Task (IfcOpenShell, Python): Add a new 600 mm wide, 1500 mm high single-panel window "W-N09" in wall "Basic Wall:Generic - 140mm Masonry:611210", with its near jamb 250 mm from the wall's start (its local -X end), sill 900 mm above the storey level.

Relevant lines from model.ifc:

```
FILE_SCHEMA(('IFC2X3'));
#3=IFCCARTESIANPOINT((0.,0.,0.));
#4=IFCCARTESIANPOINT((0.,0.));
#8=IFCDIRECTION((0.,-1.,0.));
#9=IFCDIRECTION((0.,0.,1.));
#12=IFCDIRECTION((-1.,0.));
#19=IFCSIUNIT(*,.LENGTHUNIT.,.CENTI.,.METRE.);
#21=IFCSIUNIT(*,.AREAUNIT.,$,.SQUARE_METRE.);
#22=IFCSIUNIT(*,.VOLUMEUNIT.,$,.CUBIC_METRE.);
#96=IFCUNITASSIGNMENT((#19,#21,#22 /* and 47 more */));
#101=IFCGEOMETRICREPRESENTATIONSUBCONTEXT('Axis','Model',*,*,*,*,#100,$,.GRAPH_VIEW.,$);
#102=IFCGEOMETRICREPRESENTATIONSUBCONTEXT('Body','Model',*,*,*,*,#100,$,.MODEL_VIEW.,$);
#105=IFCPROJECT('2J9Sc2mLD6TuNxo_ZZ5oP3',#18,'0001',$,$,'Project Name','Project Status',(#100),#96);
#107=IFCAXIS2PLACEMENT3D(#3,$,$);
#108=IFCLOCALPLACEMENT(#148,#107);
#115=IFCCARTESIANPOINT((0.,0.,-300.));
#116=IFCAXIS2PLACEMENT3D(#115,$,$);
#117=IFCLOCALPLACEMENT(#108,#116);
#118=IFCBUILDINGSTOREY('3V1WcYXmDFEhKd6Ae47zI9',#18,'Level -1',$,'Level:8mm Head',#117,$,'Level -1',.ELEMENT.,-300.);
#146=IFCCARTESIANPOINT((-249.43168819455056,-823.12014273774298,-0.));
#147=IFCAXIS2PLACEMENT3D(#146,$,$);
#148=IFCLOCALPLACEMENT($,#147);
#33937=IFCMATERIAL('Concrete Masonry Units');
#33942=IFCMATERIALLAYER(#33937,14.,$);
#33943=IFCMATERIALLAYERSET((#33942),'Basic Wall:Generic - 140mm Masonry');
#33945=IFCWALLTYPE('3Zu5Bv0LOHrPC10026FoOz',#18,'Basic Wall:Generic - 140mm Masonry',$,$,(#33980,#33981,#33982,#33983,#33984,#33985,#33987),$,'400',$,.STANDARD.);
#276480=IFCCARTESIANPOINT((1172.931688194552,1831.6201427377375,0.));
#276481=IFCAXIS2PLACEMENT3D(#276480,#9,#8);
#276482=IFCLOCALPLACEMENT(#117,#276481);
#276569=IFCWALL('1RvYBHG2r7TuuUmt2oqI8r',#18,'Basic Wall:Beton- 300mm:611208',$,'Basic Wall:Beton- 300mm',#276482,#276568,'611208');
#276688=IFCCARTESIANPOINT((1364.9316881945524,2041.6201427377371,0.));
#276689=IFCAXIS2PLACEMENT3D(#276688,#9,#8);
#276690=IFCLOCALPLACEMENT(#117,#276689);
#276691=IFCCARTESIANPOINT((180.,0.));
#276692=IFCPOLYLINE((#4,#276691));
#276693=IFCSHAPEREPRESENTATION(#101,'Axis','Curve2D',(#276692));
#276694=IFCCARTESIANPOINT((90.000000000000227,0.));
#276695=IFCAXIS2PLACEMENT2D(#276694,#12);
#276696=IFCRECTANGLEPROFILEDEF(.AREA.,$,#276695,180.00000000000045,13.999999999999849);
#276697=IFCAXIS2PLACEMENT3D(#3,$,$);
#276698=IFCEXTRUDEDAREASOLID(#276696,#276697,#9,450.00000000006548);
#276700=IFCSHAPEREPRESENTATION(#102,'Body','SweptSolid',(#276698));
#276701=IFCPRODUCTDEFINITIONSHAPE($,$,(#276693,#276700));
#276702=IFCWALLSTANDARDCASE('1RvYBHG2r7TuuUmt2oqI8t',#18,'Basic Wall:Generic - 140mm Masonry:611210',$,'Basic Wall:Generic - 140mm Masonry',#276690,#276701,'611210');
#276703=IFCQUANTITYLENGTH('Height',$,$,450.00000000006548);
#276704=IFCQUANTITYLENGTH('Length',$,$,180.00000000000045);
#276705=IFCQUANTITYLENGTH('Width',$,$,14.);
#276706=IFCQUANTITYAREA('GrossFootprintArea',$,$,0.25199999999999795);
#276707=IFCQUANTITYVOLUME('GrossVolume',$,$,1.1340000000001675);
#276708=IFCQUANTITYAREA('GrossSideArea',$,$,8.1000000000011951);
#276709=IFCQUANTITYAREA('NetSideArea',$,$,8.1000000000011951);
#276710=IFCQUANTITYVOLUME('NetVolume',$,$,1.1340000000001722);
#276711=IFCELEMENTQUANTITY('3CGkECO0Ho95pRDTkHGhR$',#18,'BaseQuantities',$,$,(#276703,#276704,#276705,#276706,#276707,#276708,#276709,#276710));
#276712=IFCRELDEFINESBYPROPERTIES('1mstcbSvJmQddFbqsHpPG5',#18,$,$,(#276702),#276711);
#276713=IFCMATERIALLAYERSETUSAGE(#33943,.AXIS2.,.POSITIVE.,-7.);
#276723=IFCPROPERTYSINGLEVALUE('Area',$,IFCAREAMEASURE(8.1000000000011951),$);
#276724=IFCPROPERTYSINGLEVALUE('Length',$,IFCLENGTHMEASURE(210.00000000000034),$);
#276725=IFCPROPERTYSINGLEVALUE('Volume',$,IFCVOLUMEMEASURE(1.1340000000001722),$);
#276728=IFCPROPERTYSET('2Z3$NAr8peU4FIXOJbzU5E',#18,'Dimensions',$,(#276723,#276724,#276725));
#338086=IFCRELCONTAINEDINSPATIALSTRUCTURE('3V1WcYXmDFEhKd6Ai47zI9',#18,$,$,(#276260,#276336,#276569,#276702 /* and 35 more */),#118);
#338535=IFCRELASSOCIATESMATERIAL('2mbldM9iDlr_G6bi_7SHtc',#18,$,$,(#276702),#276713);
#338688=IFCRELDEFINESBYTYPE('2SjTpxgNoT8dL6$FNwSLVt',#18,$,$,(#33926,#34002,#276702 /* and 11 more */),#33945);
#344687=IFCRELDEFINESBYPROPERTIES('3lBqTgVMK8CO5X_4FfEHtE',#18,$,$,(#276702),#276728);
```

```python
import numpy as np
import ifcopenshell
import ifcopenshell.api.feature
import ifcopenshell.api.geometry
import ifcopenshell.api.pset
import ifcopenshell.api.root
import ifcopenshell.api.spatial
import ifcopenshell.api.type
import ifcopenshell.geom
import ifcopenshell.util.element
import ifcopenshell.util.placement
import ifcopenshell.util.representation
import ifcopenshell.util.shape
import ifcopenshell.util.unit

model = ifcopenshell.open("model.ifc")
unit_scale = ifcopenshell.util.unit.calculate_unit_scale(model)
area_scale = ifcopenshell.util.unit.calculate_unit_scale(model, "AREAUNIT")
volume_scale = ifcopenshell.util.unit.calculate_unit_scale(model, "VOLUMEUNIT")
settings = ifcopenshell.geom.settings()


def volume(element):
    """Net volume in cubic metres, openings subtracted."""
    shape = ifcopenshell.geom.create_shape(settings, element)
    return ifcopenshell.util.shape.get_volume(shape.geometry)


wall = model.by_id(276702)
storey = ifcopenshell.util.element.get_container(wall, ifc_class="IfcBuildingStorey")
context = ifcopenshell.util.representation.get_context(model, "Model", "Body", "MODEL_VIEW")
before = volume(wall)

width, height, from_end, sill = 0.6, 1.5, 0.25, 0.9  # metres

# The wall runs along its own X axis, and the end named is its -X end.
wall_shape = ifcopenshell.geom.create_shape(settings, wall)
x, y, z = ifcopenshell.util.shape.get_vertices(wall_shape.geometry).T
start = x.min() + from_end
face, thickness = float(y.min()), float(y.max() - y.min())
wall_matrix = ifcopenshell.util.placement.get_local_placement(wall.ObjectPlacement)
level = ifcopenshell.util.placement.get_local_placement(storey.ObjectPlacement)[2, 3]


def in_wall(x, y):
    """Placement at x, y metres in the wall's axes, at sill height."""
    matrix = wall_matrix.copy()
    matrix[:, 3] = wall_matrix @ np.array([x / unit_scale, y / unit_scale, 0.0, 1.0])
    matrix[2, 3] = level + sill / unit_scale
    return matrix


# Opening: a box that overshoots both wall faces by 50 mm.
opening = ifcopenshell.api.root.create_entity(model, ifc_class="IfcOpeningElement")
box = ifcopenshell.api.geometry.add_wall_representation(
    model, context=context, length=width, height=height, thickness=thickness + 0.1
)
ifcopenshell.api.geometry.assign_representation(model, product=opening, representation=box)
ifcopenshell.api.geometry.edit_object_placement(model, product=opening, matrix=in_wall(start, face - 0.05), is_si=False)
ifcopenshell.api.feature.add_feature(model, feature=opening, element=wall)

window = ifcopenshell.api.root.create_entity(model, ifc_class="IfcWindow", name="W-N09")
window.OverallWidth, window.OverallHeight = width / unit_scale, height / unit_scale
body = ifcopenshell.api.geometry.add_window_representation(
    model,
    context=context,
    overall_width=window.OverallWidth,
    overall_height=window.OverallHeight,
    partition_type="SINGLE_PANEL",
)
ifcopenshell.api.geometry.assign_representation(model, product=window, representation=body)
ifcopenshell.api.spatial.assign_container(model, products=[window], relating_structure=storey)
fills = ifcopenshell.api.feature.add_filling(model, opening=opening, element=window)
fills.OwnerHistory = window.OwnerHistory  # required in IFC2X3

# IFC2X3 keeps the operation on the window style.
style = ifcopenshell.api.root.create_entity(model, ifc_class="IfcWindowStyle", name="W-N09")
style.OperationType, style.ConstructionType = "SINGLE_PANEL", "NOTDEFINED"
style.ParameterTakesPrecedence = style.Sizeable = False
ifcopenshell.api.type.assign_type(model, related_objects=[window], relating_type=style)

# Centre the window in the wall's thickness.
ifcopenshell.api.geometry.edit_object_placement(model, product=window, matrix=in_wall(start, face), is_si=False)
window_shape = ifcopenshell.geom.create_shape(settings, window)
depth = ifcopenshell.util.shape.get_vertices(window_shape.geometry)[:, 1]
offset = face + thickness / 2 - (depth.min() + depth.max()) / 2
ifcopenshell.api.geometry.edit_object_placement(model, product=window, matrix=in_wall(start, offset), is_si=False)

after = volume(wall)

# Update the wall's stored quantities.
qto = model.by_id(ifcopenshell.util.element.get_pset(wall, "BaseQuantities", should_inherit=False)["id"])
ifcopenshell.api.pset.edit_qto(model, qto=qto, properties={
    "NetSideArea": after / thickness / area_scale,
    "NetVolume": after / volume_scale,
})
pset = model.by_id(ifcopenshell.util.element.get_pset(wall, "Dimensions", should_inherit=False)["id"])
ifcopenshell.api.pset.edit_pset(model, pset=pset, properties={
    "Area": model.create_entity("IfcAreaMeasure", after / thickness / area_scale),
    "Volume": model.create_entity("IfcVolumeMeasure", after / volume_scale),
})

print(f"wall volume {before:.3f} -> {after:.3f} m3")

model.write("model-out.ifc")
```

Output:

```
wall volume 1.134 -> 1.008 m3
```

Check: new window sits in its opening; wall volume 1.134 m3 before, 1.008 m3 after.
